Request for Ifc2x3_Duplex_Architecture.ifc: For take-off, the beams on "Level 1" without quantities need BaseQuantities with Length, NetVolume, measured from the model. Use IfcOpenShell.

First a look at what the model holds.

```python
import ifcopenshell
import ifcopenshell.util.element
import ifcopenshell.util.unit

model = ifcopenshell.open("Ifc2x3_Duplex_Architecture.ifc")
print(model.schema)
for unit_type in ("LENGTHUNIT", "AREAUNIT", "VOLUMEUNIT"):
    print(unit_type, ifcopenshell.util.unit.calculate_unit_scale(model, unit_type))
storey = next(s for s in model.by_type("IfcBuildingStorey") if s.Name == "Level 1")
beams = [e for e in ifcopenshell.util.element.get_decomposition(storey) if e.is_a("IfcBeam")]
for e in sorted(beams, key=lambda e: e.id()):
    print(e.id(), e.is_a(), e.Name, list(ifcopenshell.util.element.get_psets(e, qtos_only=True)), sep=" | ")
```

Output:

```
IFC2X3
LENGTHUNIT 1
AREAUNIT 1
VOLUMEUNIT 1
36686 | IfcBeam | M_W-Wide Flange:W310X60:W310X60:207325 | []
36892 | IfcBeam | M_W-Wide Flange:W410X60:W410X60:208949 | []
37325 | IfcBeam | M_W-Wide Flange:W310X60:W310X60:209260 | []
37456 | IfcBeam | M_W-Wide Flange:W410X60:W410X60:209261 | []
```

```python
import ifcopenshell
import ifcopenshell.api.pset
import ifcopenshell.geom
import ifcopenshell.util.element
import ifcopenshell.util.shape
import ifcopenshell.util.unit

model = ifcopenshell.open("Ifc2x3_Duplex_Architecture.ifc")
unit_scale = ifcopenshell.util.unit.calculate_unit_scale(model)
volume_scale = ifcopenshell.util.unit.calculate_unit_scale(model, "VOLUMEUNIT")
settings = ifcopenshell.geom.settings()

storey = next(s for s in model.by_type("IfcBuildingStorey") if s.Name == "Level 1")
beams = [e for e in ifcopenshell.util.element.get_decomposition(storey) if e.is_a("IfcBeam")]

for e in sorted(beams, key=lambda e: e.id()):
    if ifcopenshell.util.element.get_psets(e, qtos_only=True, should_inherit=False):
        continue
    # Geometry comes back in metres, in the element's own axes.
    shape = ifcopenshell.geom.create_shape(settings, e)
    values = {
        "Length": ifcopenshell.util.shape.get_max_xyz(shape.geometry) / unit_scale,
        "NetVolume": ifcopenshell.util.shape.get_volume(shape.geometry) / volume_scale,
    }
    qto = ifcopenshell.api.pset.add_qto(model, product=e, name="BaseQuantities")
    ifcopenshell.api.pset.edit_qto(model, qto=qto, properties=values)
    print(e.id(), {k: round(v, 3) for k, v in values.items()})

model.write("Ifc2x3_Duplex_Architecture-out.ifc")
```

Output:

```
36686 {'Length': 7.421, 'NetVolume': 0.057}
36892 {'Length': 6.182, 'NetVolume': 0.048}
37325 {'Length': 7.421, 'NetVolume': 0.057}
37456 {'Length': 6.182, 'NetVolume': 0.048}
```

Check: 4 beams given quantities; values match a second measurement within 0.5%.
